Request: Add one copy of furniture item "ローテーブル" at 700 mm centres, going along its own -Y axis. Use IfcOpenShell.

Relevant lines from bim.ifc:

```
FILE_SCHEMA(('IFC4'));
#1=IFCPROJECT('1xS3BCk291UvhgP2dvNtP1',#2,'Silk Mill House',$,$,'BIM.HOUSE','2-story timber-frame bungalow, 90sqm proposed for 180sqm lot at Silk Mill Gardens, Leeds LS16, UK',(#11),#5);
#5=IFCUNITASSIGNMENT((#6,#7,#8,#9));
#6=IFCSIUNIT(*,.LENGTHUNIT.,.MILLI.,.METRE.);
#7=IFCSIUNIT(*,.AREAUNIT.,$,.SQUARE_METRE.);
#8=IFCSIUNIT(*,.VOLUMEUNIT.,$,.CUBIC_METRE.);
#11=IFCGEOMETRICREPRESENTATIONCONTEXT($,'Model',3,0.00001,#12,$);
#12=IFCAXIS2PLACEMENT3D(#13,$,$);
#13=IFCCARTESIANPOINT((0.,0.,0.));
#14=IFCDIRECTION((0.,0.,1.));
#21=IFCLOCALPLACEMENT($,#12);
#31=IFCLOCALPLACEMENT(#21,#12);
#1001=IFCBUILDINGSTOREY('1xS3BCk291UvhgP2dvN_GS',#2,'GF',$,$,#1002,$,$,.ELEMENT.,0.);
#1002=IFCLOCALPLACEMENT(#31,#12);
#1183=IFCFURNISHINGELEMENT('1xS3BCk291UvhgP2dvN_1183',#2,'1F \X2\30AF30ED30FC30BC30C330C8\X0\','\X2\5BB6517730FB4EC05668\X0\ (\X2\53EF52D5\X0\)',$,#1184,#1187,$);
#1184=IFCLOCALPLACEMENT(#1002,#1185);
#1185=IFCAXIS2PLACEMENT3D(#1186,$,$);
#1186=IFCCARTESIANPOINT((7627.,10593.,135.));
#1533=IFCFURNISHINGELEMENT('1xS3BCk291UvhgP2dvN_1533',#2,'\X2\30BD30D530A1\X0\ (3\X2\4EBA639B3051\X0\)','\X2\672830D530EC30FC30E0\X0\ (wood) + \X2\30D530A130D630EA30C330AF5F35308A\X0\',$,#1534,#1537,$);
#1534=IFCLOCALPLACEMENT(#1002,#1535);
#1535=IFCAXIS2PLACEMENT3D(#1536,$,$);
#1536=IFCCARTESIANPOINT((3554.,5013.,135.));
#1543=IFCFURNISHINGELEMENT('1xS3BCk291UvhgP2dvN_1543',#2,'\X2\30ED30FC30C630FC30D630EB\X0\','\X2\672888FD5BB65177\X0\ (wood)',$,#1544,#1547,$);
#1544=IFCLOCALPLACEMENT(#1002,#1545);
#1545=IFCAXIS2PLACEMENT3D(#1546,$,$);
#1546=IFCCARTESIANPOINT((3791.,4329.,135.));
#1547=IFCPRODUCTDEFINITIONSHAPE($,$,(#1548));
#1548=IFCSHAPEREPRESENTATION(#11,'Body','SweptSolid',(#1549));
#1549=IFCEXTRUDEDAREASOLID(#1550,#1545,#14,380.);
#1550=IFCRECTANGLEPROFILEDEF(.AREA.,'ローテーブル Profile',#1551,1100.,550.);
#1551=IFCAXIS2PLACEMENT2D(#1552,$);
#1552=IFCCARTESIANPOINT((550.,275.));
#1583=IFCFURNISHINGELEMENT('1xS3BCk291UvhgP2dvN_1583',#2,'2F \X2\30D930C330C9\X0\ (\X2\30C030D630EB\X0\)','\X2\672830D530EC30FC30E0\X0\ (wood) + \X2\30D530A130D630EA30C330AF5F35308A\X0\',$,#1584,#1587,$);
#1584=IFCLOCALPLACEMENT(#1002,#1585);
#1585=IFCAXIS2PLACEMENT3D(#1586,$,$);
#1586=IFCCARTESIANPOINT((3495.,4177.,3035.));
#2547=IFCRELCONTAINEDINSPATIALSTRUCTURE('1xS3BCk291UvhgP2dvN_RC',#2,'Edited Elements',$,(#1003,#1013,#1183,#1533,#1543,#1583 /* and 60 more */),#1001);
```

```python
import ifcopenshell
import ifcopenshell.api.geometry
import ifcopenshell.api.root
import ifcopenshell.util.element
import ifcopenshell.util.placement
import ifcopenshell.util.unit

model = ifcopenshell.open("bim.ifc")
unit_scale = ifcopenshell.util.unit.calculate_unit_scale(model)


def reuse_history(source, copy):
    """copy_class also copies each property set's owner history, people and application; keep the originals."""
    for rel in copy.IsDefinedBy:
        if rel.is_a("IfcRelDefinesByProperties") and (history := rel.RelatingPropertyDefinition.OwnerHistory):
            rel.RelatingPropertyDefinition.OwnerHistory = source.OwnerHistory
            ifcopenshell.util.element.remove_deep2(model, history)


source = model.by_guid("1xS3BCk291UvhgP2dvN_1543")
base = ifcopenshell.util.placement.get_local_placement(source.ObjectPlacement)
step = -base[:3, 1] * 0.7 / unit_scale

for i in range(1, 2):
    copy = ifcopenshell.api.root.copy_class(model, product=source)
    copy.Representation = ifcopenshell.util.element.copy_deep(
        model, source.Representation, exclude=["IfcGeometricRepresentationContext", "IfcRepresentationMap"]
    )
    reuse_history(source, copy)
    matrix = base.copy()
    matrix[:3, 3] += i * step
    print("added at", matrix[:3, 3].round(3) + 0.0)
    ifcopenshell.api.geometry.edit_object_placement(model, product=copy, matrix=matrix, is_si=False)

model.write("bim_edited.ifc")
```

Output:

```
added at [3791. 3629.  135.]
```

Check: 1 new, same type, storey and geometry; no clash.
